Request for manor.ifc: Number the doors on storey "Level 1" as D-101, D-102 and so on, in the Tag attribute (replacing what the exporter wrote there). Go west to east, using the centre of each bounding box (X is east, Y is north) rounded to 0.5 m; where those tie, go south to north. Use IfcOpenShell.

First a look at what the model holds.

```python
import ifcopenshell
import ifcopenshell.util.element
import ifcopenshell.util.placement

model = ifcopenshell.open("manor.ifc")
print(model.schema)
storey = next(s for s in model.by_type("IfcBuildingStorey") if s.Name == "Level 1")
doors = [e for e in ifcopenshell.util.element.get_decomposition(storey) if e.is_a("IfcDoor")]
for e in sorted(doors, key=lambda e: e.id()):
    origin = ifcopenshell.util.placement.get_local_placement(e.ObjectPlacement)[:3, 3]
    print(e.id(), e.Tag, e.Name, origin.round(2) + 0.0, sep=" | ")
```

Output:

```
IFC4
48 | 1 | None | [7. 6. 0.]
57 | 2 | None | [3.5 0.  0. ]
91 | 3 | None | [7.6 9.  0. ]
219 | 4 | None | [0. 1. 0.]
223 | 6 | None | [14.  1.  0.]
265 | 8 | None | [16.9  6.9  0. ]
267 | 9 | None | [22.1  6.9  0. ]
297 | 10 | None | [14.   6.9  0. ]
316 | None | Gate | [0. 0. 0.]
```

```python
import ifcopenshell
import ifcopenshell.geom
import ifcopenshell.util.element
import ifcopenshell.util.shape

model = ifcopenshell.open("manor.ifc")
settings = ifcopenshell.geom.settings()
settings.set("use-world-coords", True)


def centre(element):
    shape = ifcopenshell.geom.create_shape(settings, element)
    return ifcopenshell.util.shape.get_bbox_centroid(shape.geometry)


storey = next(s for s in model.by_type("IfcBuildingStorey") if s.Name == "Level 1")
doors = [e for e in ifcopenshell.util.element.get_decomposition(storey) if e.is_a("IfcDoor")]

# Insertion points can sit at a corner or the storey origin, so sort by the geometry (in metres).
centres = {e: centre(e) for e in doors}
doors.sort(key=lambda e: (round(centres[e][0] / 0.5), centres[e][1]))

for i, e in enumerate(doors, start=1):
    number = f"D-1{i:02d}"
    e.Tag = number
    print(e.id(), number)

model.write("manor-out.ifc")
```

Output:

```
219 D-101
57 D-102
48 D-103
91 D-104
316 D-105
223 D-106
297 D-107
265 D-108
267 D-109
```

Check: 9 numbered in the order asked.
